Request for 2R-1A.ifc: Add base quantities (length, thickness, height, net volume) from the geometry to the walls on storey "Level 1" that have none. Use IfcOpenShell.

First a look at what the model holds.

```python
import ifcopenshell
import ifcopenshell.util.element
import ifcopenshell.util.unit

model = ifcopenshell.open("2R-1A.ifc")
print(model.schema)
for unit_type in ("LENGTHUNIT", "AREAUNIT", "VOLUMEUNIT"):
    print(unit_type, ifcopenshell.util.unit.calculate_unit_scale(model, unit_type))
storey = next(s for s in model.by_type("IfcBuildingStorey") if s.Name == "Level 1")
walls = [e for e in ifcopenshell.util.element.get_decomposition(storey) if e.is_a("IfcWall")]
for e in sorted(walls, key=lambda e: e.id()):
    print(e.id(), e.is_a(), e.Name, list(ifcopenshell.util.element.get_psets(e, qtos_only=True)), sep=" | ")
```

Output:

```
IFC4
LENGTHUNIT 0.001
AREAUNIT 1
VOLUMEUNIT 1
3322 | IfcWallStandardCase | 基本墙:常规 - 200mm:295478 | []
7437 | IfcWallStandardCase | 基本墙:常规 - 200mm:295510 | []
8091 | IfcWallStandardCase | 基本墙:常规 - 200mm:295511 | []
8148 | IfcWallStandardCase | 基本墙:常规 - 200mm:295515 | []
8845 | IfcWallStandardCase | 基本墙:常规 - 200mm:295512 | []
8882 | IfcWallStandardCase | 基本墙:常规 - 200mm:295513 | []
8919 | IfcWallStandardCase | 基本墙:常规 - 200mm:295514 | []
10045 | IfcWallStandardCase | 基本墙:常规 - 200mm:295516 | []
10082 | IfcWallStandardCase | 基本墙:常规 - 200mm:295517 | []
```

```python
import ifcopenshell
import ifcopenshell.api.pset
import ifcopenshell.geom
import ifcopenshell.util.element
import ifcopenshell.util.shape
import ifcopenshell.util.unit

model = ifcopenshell.open("2R-1A.ifc")
unit_scale = ifcopenshell.util.unit.calculate_unit_scale(model)
volume_scale = ifcopenshell.util.unit.calculate_unit_scale(model, "VOLUMEUNIT")
settings = ifcopenshell.geom.settings()

storey = next(s for s in model.by_type("IfcBuildingStorey") if s.Name == "Level 1")
walls = [e for e in ifcopenshell.util.element.get_decomposition(storey) if e.is_a("IfcWall")]

for e in sorted(walls, key=lambda e: e.id()):
    if ifcopenshell.util.element.get_psets(e, qtos_only=True, should_inherit=False):
        continue
    # Geometry comes back in metres, in the element's own axes.
    shape = ifcopenshell.geom.create_shape(settings, e)
    values = {
        "Length": ifcopenshell.util.shape.get_x(shape.geometry) / unit_scale,
        "Width": ifcopenshell.util.shape.get_y(shape.geometry) / unit_scale,
        "Height": ifcopenshell.util.shape.get_z(shape.geometry) / unit_scale,
        "NetVolume": ifcopenshell.util.shape.get_volume(shape.geometry) / volume_scale,
    }
    qto = ifcopenshell.api.pset.add_qto(model, product=e, name="Qto_WallBaseQuantities")
    ifcopenshell.api.pset.edit_qto(model, qto=qto, properties=values)
    print(e.id(), {k: round(v, 3) for k, v in values.items()})

model.write("2R-1A-out.ifc")
```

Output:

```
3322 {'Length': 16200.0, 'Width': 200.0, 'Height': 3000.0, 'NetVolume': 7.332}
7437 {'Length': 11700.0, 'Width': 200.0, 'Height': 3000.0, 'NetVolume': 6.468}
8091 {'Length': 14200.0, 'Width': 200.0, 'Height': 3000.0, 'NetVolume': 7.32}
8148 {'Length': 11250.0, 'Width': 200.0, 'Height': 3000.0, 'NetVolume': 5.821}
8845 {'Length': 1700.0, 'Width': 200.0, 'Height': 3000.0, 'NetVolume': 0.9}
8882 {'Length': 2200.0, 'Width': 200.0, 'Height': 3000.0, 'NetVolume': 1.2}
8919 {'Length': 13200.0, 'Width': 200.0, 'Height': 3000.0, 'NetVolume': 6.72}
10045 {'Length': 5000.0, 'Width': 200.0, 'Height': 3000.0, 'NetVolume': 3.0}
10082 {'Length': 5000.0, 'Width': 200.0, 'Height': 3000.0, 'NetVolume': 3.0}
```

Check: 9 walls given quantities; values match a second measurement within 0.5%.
